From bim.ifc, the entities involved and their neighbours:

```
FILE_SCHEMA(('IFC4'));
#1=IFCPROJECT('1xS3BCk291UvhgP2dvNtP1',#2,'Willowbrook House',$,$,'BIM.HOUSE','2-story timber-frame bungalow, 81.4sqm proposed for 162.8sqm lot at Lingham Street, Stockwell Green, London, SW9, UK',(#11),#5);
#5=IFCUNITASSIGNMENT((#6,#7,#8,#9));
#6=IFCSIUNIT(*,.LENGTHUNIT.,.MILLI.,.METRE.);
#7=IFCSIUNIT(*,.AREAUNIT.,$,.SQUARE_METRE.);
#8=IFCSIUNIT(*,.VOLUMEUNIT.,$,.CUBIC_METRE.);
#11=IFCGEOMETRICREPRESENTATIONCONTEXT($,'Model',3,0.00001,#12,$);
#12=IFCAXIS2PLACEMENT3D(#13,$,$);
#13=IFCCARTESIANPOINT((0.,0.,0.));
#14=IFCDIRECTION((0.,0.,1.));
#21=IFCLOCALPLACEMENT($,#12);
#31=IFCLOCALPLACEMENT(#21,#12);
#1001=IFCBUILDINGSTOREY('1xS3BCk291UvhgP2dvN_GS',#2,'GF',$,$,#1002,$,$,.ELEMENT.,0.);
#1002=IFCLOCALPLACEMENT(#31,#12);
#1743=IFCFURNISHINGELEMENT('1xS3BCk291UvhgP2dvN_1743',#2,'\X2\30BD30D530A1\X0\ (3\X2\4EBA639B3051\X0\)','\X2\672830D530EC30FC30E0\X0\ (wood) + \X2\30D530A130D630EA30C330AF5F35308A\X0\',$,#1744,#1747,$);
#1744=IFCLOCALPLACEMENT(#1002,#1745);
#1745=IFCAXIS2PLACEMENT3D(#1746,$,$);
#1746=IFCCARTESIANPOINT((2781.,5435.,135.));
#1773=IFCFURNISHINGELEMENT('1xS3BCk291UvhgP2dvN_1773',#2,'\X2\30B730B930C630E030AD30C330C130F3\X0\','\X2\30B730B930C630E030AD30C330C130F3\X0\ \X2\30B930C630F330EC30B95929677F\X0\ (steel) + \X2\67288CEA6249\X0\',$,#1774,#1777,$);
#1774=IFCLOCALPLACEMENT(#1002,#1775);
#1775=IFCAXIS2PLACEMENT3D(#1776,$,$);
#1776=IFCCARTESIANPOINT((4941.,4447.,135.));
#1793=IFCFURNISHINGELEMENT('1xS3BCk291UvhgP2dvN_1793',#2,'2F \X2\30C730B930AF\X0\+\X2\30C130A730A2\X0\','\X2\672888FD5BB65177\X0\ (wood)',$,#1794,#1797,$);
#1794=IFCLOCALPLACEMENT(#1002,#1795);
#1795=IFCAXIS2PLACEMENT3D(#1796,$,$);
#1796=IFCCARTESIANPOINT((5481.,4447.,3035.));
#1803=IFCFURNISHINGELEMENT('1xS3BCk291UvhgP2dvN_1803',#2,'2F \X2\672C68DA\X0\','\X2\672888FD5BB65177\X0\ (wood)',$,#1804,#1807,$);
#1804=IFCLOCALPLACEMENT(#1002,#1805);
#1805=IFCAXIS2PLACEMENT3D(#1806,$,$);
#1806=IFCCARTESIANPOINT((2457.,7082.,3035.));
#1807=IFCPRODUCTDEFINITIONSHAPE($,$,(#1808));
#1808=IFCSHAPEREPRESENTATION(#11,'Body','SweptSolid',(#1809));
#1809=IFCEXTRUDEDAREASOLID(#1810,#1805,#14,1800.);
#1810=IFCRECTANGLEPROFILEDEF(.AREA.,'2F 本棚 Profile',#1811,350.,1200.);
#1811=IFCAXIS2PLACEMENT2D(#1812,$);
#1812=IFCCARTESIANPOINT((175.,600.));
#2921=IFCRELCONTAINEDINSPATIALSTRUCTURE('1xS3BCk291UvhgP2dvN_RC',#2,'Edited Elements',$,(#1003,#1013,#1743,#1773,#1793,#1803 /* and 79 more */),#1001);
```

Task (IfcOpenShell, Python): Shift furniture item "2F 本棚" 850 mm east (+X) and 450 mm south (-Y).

```python
import ifcopenshell
import ifcopenshell.api.geometry
import ifcopenshell.util.placement

model = ifcopenshell.open("bim.ifc")

item = model.by_guid("1xS3BCk291UvhgP2dvN_1803")
matrix = ifcopenshell.util.placement.get_local_placement(item.ObjectPlacement)
matrix[0, 3] += 850.0
matrix[1, 3] -= 450.0
ifcopenshell.api.geometry.edit_object_placement(model, product=item, matrix=matrix, is_si=False)

print(ifcopenshell.util.placement.get_local_placement(item.ObjectPlacement).round(3) + 0.0)

model.write("bim_edited.ifc")
```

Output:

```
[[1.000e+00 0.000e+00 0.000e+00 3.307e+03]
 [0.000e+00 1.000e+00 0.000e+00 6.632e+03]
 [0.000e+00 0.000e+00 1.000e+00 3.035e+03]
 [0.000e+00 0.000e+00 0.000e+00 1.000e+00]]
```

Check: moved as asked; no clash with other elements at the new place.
